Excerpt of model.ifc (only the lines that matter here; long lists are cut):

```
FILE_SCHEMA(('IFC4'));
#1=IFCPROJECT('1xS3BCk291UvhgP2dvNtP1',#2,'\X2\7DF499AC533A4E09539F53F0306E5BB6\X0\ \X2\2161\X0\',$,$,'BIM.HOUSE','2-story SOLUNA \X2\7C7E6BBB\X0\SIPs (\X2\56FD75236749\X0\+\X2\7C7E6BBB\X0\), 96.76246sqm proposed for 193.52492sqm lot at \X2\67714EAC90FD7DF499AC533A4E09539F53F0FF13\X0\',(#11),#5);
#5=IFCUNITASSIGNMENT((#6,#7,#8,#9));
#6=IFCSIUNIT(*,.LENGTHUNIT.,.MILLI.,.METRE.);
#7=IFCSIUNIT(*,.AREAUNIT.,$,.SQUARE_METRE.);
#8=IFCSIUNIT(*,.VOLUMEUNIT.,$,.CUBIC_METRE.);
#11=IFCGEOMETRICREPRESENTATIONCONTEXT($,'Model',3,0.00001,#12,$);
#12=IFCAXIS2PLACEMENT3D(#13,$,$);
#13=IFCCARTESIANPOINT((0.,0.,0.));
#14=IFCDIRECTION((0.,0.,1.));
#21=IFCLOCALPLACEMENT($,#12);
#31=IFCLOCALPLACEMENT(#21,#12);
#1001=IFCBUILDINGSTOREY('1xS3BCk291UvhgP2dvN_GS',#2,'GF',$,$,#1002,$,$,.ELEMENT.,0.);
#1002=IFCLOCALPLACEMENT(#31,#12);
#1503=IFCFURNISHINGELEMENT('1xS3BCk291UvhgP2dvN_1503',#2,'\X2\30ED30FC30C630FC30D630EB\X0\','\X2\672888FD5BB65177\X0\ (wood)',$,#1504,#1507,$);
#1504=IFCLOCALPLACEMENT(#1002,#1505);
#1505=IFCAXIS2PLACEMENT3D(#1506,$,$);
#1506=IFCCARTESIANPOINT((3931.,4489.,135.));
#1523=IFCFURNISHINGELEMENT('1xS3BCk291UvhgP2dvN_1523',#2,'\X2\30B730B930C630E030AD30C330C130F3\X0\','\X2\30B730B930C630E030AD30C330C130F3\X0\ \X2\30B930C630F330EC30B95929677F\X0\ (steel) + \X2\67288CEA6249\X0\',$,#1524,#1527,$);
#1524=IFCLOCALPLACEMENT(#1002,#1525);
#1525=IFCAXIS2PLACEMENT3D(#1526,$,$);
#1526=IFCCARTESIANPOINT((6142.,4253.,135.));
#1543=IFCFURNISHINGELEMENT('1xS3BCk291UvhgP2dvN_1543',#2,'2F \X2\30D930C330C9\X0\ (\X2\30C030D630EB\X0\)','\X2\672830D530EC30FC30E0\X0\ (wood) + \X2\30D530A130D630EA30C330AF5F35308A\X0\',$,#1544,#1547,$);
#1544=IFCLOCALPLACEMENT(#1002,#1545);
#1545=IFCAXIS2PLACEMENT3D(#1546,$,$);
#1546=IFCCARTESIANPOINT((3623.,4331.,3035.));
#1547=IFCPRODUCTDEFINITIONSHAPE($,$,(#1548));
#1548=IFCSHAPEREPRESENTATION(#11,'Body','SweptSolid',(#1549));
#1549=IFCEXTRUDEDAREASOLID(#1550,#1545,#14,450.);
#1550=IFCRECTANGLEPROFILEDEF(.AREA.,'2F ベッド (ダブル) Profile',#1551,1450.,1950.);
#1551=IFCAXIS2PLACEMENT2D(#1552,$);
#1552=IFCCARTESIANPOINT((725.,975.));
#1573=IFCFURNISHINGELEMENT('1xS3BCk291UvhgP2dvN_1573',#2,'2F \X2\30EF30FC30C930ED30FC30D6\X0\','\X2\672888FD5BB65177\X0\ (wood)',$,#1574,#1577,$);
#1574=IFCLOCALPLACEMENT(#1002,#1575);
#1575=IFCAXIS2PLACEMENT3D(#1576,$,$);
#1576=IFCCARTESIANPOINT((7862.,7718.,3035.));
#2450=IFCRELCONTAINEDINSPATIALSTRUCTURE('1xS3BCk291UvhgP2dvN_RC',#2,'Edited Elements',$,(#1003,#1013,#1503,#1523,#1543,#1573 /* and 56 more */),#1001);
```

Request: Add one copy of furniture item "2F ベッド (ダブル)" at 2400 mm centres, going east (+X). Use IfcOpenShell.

```python
import numpy as np
import ifcopenshell
import ifcopenshell.api.geometry
import ifcopenshell.api.root
import ifcopenshell.util.element
import ifcopenshell.util.placement
import ifcopenshell.util.unit

model = ifcopenshell.open("model.ifc")
unit_scale = ifcopenshell.util.unit.calculate_unit_scale(model)


def reuse_history(source, copy):
    """copy_class also copies each property set's owner history, people and application; keep the originals."""
    for rel in copy.IsDefinedBy:
        if rel.is_a("IfcRelDefinesByProperties") and (history := rel.RelatingPropertyDefinition.OwnerHistory):
            rel.RelatingPropertyDefinition.OwnerHistory = source.OwnerHistory
            ifcopenshell.util.element.remove_deep2(model, history)


source = model.by_guid("1xS3BCk291UvhgP2dvN_1543")
base = ifcopenshell.util.placement.get_local_placement(source.ObjectPlacement)
step = np.array([1.0, 0.0, 0.0]) * 2.4 / unit_scale

for i in range(1, 2):
    copy = ifcopenshell.api.root.copy_class(model, product=source)
    copy.Representation = ifcopenshell.util.element.copy_deep(
        model, source.Representation, exclude=["IfcGeometricRepresentationContext", "IfcRepresentationMap"]
    )
    reuse_history(source, copy)
    matrix = base.copy()
    matrix[:3, 3] += i * step
    print("added at", matrix[:3, 3].round(3) + 0.0)
    ifcopenshell.api.geometry.edit_object_placement(model, product=copy, matrix=matrix, is_si=False)

model.write("model_rev.ifc")
```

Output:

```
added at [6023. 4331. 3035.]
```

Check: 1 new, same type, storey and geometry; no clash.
